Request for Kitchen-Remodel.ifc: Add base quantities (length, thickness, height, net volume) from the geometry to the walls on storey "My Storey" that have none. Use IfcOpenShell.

First a look at what the model holds.

```python
import ifcopenshell
import ifcopenshell.util.element
import ifcopenshell.util.unit

model = ifcopenshell.open("Kitchen-Remodel.ifc")
print(model.schema)
for unit_type in ("LENGTHUNIT", "AREAUNIT", "VOLUMEUNIT"):
    print(unit_type, ifcopenshell.util.unit.calculate_unit_scale(model, unit_type))
storey = next(s for s in model.by_type("IfcBuildingStorey") if s.Name == "My Storey")
walls = [e for e in ifcopenshell.util.element.get_decomposition(storey) if e.is_a("IfcWall")]
for e in sorted(walls, key=lambda e: e.id()):
    print(e.id(), e.is_a(), e.Name, list(ifcopenshell.util.element.get_psets(e, qtos_only=True)), sep=" | ")
```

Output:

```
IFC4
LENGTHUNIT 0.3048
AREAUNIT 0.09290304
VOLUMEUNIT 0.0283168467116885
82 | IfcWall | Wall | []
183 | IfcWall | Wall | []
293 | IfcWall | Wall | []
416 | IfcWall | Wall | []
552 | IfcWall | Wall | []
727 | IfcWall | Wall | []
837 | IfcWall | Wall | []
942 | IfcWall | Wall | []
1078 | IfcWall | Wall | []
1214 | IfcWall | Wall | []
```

```python
import ifcopenshell
import ifcopenshell.api.pset
import ifcopenshell.geom
import ifcopenshell.util.element
import ifcopenshell.util.shape
import ifcopenshell.util.unit

model = ifcopenshell.open("Kitchen-Remodel.ifc")
unit_scale = ifcopenshell.util.unit.calculate_unit_scale(model)
volume_scale = ifcopenshell.util.unit.calculate_unit_scale(model, "VOLUMEUNIT")
settings = ifcopenshell.geom.settings()

storey = next(s for s in model.by_type("IfcBuildingStorey") if s.Name == "My Storey")
walls = [e for e in ifcopenshell.util.element.get_decomposition(storey) if e.is_a("IfcWall")]

for e in sorted(walls, key=lambda e: e.id()):
    if ifcopenshell.util.element.get_psets(e, qtos_only=True, should_inherit=False):
        continue
    # Geometry comes back in metres, in the element's own axes.
    shape = ifcopenshell.geom.create_shape(settings, e)
    values = {
        "Length": ifcopenshell.util.shape.get_x(shape.geometry) / unit_scale,
        "Width": ifcopenshell.util.shape.get_y(shape.geometry) / unit_scale,
        "Height": ifcopenshell.util.shape.get_z(shape.geometry) / unit_scale,
        "NetVolume": ifcopenshell.util.shape.get_volume(shape.geometry) / volume_scale,
    }
    qto = ifcopenshell.api.pset.add_qto(model, product=e, name="Qto_WallBaseQuantities")
    ifcopenshell.api.pset.edit_qto(model, qto=qto, properties=values)
    print(e.id(), {k: round(v, 3) for k, v in values.items()})

model.write("Kitchen-Remodel-out.ifc")
```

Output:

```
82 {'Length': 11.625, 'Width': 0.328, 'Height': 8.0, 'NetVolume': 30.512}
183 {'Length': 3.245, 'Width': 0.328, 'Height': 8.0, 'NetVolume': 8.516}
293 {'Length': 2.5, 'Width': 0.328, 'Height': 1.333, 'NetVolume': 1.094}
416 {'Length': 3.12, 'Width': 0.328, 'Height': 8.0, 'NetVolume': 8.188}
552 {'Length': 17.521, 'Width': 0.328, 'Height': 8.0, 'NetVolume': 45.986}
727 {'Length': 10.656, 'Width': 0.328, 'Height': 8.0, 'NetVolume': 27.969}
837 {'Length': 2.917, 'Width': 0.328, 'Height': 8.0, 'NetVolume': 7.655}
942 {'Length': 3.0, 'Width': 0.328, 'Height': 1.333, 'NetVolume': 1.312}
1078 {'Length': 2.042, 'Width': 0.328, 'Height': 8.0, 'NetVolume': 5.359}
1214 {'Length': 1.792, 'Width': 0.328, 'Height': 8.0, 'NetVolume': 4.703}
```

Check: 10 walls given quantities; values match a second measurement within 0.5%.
